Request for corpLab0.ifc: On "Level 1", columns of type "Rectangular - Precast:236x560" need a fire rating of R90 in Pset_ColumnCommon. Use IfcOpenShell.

First a look at what the model holds.

```python
import ifcopenshell
import ifcopenshell.util.element

model = ifcopenshell.open("corpLab0.ifc")
print(model.schema)
storey = next(s for s in model.by_type("IfcBuildingStorey") if s.Name == "Level 1")
columns = [e for e in ifcopenshell.util.element.get_decomposition(storey) if e.is_a("IfcColumn")]
seen = {}
for e in columns:
    element_type = ifcopenshell.util.element.get_type(e)
    key = (element_type.Name if element_type != e and element_type else None, ifcopenshell.util.element.get_pset(e, "Pset_ColumnCommon", "FireRating"))
    seen[key] = seen.get(key, 0) + 1
for (name, value), count in sorted(seen.items(), key=str):
    print(count, "x", name, "|", value)
```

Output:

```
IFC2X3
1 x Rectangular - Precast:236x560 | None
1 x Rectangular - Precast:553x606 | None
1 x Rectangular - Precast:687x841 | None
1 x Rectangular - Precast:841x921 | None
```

```python
import ifcopenshell
import ifcopenshell.api.pset
import ifcopenshell.util.element

model = ifcopenshell.open("corpLab0.ifc")

storey = next(s for s in model.by_type("IfcBuildingStorey") if s.Name == "Level 1")
columns = [e for e in ifcopenshell.util.element.get_decomposition(storey) if e.is_a("IfcColumn")]

count = 0
for e in columns:
    element_type = ifcopenshell.util.element.get_type(e)
    if element_type in (None, e) or element_type.Name != "Rectangular - Precast:236x560":
        continue
    # add_pset returns the element's existing set when there is one.
    pset = ifcopenshell.api.pset.add_pset(model, product=e, name="Pset_ColumnCommon")
    ifcopenshell.api.pset.edit_pset(model, pset=pset, properties={"FireRating": "R90"})
    count += 1

print(count, "columns updated")

model.write("corpLab0_rev.ifc")
```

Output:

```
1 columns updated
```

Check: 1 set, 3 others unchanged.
